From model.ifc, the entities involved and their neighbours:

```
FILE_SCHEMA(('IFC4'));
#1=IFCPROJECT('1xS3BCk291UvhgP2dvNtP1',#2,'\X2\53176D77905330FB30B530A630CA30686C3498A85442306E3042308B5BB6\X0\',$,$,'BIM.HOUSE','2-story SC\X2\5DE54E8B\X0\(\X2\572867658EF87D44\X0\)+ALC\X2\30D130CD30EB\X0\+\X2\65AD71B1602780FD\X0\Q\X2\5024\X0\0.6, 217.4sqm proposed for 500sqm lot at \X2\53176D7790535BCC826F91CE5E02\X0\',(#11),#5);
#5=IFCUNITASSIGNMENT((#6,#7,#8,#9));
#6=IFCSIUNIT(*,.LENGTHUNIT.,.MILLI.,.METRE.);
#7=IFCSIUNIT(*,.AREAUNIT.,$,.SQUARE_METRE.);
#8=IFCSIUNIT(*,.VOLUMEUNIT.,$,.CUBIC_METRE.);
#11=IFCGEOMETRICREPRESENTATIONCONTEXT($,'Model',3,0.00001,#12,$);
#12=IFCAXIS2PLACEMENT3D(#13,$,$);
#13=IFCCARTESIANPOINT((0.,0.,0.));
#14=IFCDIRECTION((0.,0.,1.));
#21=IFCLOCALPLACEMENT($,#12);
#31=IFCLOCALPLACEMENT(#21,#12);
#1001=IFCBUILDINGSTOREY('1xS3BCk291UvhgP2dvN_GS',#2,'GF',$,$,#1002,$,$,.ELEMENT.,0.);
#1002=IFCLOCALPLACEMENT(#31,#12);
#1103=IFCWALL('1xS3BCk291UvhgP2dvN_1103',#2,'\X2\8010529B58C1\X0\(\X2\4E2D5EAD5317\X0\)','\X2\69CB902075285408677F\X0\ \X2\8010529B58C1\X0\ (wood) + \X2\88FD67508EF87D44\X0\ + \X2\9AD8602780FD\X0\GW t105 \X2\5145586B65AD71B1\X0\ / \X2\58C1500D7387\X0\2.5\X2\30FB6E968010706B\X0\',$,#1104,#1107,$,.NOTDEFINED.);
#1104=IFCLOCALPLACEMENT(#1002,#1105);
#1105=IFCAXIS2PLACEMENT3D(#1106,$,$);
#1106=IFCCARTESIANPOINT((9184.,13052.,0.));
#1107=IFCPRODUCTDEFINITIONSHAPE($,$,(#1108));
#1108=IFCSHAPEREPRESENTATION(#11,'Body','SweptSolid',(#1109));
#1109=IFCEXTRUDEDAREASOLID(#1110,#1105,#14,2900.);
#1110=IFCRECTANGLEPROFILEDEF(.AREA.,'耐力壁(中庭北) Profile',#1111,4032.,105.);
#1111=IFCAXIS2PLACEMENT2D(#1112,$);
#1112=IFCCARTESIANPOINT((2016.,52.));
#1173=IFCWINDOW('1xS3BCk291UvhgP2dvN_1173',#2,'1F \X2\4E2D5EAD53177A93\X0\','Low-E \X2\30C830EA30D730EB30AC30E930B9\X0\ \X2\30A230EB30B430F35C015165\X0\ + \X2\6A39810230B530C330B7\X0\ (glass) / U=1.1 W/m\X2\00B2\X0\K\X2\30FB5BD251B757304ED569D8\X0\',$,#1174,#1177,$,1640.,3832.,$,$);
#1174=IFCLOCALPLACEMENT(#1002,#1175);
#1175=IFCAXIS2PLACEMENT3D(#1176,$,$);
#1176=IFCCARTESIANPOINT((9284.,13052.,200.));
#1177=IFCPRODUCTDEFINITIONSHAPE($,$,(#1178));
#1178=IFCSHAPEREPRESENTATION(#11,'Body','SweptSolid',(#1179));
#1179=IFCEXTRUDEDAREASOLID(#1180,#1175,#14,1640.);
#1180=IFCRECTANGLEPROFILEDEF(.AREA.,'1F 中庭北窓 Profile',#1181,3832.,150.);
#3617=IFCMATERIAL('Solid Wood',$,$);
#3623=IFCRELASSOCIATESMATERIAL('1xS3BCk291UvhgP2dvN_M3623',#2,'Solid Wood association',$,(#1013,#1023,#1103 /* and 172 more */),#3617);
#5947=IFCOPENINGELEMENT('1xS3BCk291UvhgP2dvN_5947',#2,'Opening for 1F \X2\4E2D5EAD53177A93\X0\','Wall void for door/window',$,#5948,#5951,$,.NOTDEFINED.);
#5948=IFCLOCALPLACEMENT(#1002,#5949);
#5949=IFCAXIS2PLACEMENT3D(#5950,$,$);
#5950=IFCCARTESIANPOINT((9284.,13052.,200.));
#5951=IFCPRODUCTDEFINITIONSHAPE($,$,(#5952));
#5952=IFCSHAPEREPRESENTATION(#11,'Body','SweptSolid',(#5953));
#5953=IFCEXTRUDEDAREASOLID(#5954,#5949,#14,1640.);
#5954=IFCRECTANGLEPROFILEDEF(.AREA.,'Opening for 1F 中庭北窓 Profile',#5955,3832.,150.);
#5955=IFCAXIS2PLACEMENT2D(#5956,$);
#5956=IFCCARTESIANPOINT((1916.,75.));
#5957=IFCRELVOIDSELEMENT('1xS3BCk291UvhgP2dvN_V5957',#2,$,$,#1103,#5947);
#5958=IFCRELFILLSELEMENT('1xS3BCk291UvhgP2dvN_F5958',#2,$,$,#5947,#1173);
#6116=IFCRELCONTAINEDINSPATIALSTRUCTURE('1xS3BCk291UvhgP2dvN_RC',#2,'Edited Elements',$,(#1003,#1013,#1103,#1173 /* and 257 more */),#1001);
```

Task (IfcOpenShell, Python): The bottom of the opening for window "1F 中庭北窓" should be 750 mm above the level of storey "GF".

```python
import numpy as np
import ifcopenshell
import ifcopenshell.api.geometry
import ifcopenshell.geom
import ifcopenshell.util.element
import ifcopenshell.util.placement
import ifcopenshell.util.shape
import ifcopenshell.util.unit

model = ifcopenshell.open("model.ifc")
unit_scale = ifcopenshell.util.unit.calculate_unit_scale(model)

window = model.by_guid("1xS3BCk291UvhgP2dvN_1173")
opening = window.FillsVoids[0].RelatingOpeningElement
storey = ifcopenshell.util.element.get_container(window, ifc_class="IfcBuildingStorey")
level = ifcopenshell.util.placement.get_local_placement(storey.ObjectPlacement)[2, 3]

# The opening's origin need not be at the sill, so measure its lowest point.
shape = ifcopenshell.geom.create_shape(ifcopenshell.geom.settings(), opening)
bottom = ifcopenshell.util.shape.get_shape_bottom_elevation(shape, shape.geometry) / unit_scale
dz = level + 0.75 / unit_scale - bottom

shift = np.array([0.0, 0.0, dz])
# The window is not placed relative to its opening, so move both.
for product in (opening, window):
    matrix = ifcopenshell.util.placement.get_local_placement(product.ObjectPlacement)
    matrix[:3, 3] += shift
    ifcopenshell.api.geometry.edit_object_placement(model, product=product, matrix=matrix, is_si=False)

print(f"moved by {dz * unit_scale:+.3f} m")

model.write("model_rev.ifc")
```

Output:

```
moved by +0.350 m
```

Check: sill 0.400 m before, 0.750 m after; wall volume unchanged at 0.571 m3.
